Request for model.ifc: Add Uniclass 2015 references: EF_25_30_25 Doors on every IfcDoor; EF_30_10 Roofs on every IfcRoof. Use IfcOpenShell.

First a look at what the model holds.

```python
import ifcopenshell

model = ifcopenshell.open("model.ifc")
print(model.schema)
print("classifications:", [c.Name for c in model.by_type("IfcClassification")])
for ifc_class in ("IfcDoor", "IfcRoof", "IfcStair", "IfcWall", "IfcWindow"):
    print(ifc_class, len(model.by_type(ifc_class)))
```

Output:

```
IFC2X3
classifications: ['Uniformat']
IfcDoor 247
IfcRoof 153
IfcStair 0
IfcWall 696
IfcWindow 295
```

```python
import ifcopenshell
import ifcopenshell.api.classification

model = ifcopenshell.open("model.ifc")

# IFC2X3 requires Source and Edition and has no link from the project to the system.
system = model.create_entity("IfcClassification", Source="NBS", Edition="2015", Name="Uniclass 2015")

codes = {
    "IfcDoor": ("EF_25_30_25", "Doors"),
    "IfcRoof": ("EF_30_10", "Roofs"),
}
for ifc_class, (code, name) in codes.items():
    products = model.by_type(ifc_class)
    ifcopenshell.api.classification.add_reference(
        model, products=products, classification=system, identification=code, name=name
    )
    print(code, len(products))

model.write("model_v2.ifc")
```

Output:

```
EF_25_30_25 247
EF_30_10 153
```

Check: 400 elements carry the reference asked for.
